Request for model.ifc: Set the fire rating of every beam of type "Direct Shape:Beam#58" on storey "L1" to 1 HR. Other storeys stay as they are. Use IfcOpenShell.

First a look at what the model holds.

```python
import ifcopenshell
import ifcopenshell.util.element

model = ifcopenshell.open("model.ifc")
print(model.schema)
storey = next(s for s in model.by_type("IfcBuildingStorey") if s.Name == "L1")
beams = [e for e in ifcopenshell.util.element.get_decomposition(storey) if e.is_a("IfcBeam")]
seen = {}
for e in beams:
    element_type = ifcopenshell.util.element.get_type(e)
    key = (element_type.Name if element_type != e and element_type else None, ifcopenshell.util.element.get_pset(e, "Pset_BeamCommon", "FireRating"))
    seen[key] = seen.get(key, 0) + 1
for (name, value), count in sorted(seen.items(), key=str):
    print(count, "x", name, "|", value)
```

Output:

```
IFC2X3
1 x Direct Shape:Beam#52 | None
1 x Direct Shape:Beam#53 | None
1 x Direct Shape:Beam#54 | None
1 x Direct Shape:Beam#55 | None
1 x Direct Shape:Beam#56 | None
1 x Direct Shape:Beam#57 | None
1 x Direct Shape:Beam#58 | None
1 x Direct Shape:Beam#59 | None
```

```python
import ifcopenshell
import ifcopenshell.api.pset
import ifcopenshell.util.element

model = ifcopenshell.open("model.ifc")

storey = next(s for s in model.by_type("IfcBuildingStorey") if s.Name == "L1")
beams = [e for e in ifcopenshell.util.element.get_decomposition(storey) if e.is_a("IfcBeam")]

count = 0
for e in beams:
    element_type = ifcopenshell.util.element.get_type(e)
    if element_type in (None, e) or element_type.Name != "Direct Shape:Beam#58":
        continue
    # add_pset returns the element's existing set when there is one.
    pset = ifcopenshell.api.pset.add_pset(model, product=e, name="Pset_BeamCommon")
    ifcopenshell.api.pset.edit_pset(model, pset=pset, properties={"FireRating": "1 HR"})
    count += 1

print(count, "beams updated")

model.write("model_updated.ifc")
```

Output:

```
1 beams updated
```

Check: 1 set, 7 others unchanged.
